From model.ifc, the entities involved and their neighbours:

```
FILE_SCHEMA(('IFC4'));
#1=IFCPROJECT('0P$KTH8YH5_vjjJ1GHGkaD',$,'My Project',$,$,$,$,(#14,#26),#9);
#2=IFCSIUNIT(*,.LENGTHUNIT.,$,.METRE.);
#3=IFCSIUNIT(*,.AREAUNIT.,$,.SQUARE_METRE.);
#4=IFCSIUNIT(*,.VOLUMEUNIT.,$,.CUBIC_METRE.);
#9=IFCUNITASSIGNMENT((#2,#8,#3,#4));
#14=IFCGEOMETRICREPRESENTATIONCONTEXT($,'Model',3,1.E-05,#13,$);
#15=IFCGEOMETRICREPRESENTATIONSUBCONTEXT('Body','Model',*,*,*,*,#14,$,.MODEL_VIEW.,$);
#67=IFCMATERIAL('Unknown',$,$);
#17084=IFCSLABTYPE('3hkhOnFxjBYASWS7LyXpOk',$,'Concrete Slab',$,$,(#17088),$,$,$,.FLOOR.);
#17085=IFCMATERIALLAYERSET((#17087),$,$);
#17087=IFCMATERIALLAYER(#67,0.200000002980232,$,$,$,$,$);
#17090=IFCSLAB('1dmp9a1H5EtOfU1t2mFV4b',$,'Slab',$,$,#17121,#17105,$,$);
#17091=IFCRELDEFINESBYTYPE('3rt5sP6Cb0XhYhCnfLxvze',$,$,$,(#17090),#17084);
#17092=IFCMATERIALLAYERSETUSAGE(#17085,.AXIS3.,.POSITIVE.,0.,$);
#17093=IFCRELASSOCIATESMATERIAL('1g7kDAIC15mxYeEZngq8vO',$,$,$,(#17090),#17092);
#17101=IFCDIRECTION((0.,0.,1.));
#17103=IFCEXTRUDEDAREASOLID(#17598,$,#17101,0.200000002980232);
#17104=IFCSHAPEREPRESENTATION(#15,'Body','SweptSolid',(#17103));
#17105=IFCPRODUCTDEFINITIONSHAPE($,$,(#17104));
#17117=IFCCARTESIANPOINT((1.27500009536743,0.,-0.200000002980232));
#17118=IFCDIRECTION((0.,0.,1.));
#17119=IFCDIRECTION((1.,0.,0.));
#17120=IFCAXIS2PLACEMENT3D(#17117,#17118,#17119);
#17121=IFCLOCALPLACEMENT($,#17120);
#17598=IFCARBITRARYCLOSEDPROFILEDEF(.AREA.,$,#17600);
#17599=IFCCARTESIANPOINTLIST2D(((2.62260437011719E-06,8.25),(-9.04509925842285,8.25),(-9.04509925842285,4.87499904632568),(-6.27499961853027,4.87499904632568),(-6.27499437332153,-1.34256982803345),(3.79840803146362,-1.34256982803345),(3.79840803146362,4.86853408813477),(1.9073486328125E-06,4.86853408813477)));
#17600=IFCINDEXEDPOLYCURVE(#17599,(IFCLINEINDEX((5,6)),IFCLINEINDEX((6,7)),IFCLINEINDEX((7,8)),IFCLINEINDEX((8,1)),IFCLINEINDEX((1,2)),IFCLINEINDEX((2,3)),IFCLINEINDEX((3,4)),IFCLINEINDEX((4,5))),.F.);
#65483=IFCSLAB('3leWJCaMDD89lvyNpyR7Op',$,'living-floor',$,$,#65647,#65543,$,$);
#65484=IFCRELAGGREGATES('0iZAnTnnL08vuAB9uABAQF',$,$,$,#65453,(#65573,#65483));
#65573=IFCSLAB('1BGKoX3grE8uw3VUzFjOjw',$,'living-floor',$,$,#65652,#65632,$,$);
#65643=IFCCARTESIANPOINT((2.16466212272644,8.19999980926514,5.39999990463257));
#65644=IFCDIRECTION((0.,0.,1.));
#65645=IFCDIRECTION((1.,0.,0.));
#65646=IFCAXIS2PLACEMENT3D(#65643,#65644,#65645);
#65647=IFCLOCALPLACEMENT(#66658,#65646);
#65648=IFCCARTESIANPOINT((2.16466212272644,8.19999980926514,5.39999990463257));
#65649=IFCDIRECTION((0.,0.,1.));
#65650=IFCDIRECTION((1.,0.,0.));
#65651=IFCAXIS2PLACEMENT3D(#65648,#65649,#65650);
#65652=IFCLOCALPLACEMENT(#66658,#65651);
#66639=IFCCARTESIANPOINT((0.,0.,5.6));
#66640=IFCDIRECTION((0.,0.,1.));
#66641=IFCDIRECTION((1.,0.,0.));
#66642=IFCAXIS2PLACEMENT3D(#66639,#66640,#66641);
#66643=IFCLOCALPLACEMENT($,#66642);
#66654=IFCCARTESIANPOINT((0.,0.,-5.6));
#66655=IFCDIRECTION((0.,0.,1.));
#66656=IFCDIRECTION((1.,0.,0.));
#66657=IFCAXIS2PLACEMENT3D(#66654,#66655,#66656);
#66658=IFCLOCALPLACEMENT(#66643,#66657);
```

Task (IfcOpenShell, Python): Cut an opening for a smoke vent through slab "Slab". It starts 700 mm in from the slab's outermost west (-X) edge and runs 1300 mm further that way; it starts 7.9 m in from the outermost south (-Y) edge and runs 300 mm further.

```python
import numpy as np
import ifcopenshell
import ifcopenshell.api.feature
import ifcopenshell.api.geometry
import ifcopenshell.api.root
import ifcopenshell.geom
import ifcopenshell.util.placement
import ifcopenshell.util.representation
import ifcopenshell.util.shape
import ifcopenshell.util.unit

model = ifcopenshell.open("model.ifc")
unit_scale = ifcopenshell.util.unit.calculate_unit_scale(model)
settings = ifcopenshell.geom.settings()


def volume(element):
    """Net volume in cubic metres, openings subtracted."""
    shape = ifcopenshell.geom.create_shape(settings, element)
    return ifcopenshell.util.shape.get_volume(shape.geometry)


slab = model.by_guid("1dmp9a1H5EtOfU1t2mFV4b")
before = volume(slab)

# Extent in the slab's own axes, in metres. The edges named are its -X and -Y sides.
slab_shape = ifcopenshell.geom.create_shape(settings, slab)
vertices = ifcopenshell.util.shape.get_vertices(slab_shape.geometry)
x_min, y_min, bottom = vertices.min(axis=0)
top = vertices[:, 2].max()

opening = ifcopenshell.api.root.create_entity(model, ifc_class="IfcOpeningElement", name="Smoke vent opening", predefined_type="OPENING")
context = ifcopenshell.util.representation.get_context(model, "Model", "Body", "MODEL_VIEW")
width, depth = 1.3, 0.3
outline = [(0.0, 0.0), (width, 0.0), (width, depth), (0.0, depth), (0.0, 0.0)]
# Overshoot both faces by 50 mm so the cut is clean.
shape = ifcopenshell.api.geometry.add_slab_representation(
    model, context=context, depth=top - bottom + 0.1, polyline=outline
)
ifcopenshell.api.geometry.assign_representation(model, product=opening, representation=shape)

matrix = ifcopenshell.util.placement.get_local_placement(slab.ObjectPlacement)
matrix[:, 3] = matrix @ np.append(np.array([x_min + 0.7, y_min + 7.9, bottom - 0.05]) / unit_scale, 1.0)
ifcopenshell.api.geometry.edit_object_placement(model, product=opening, matrix=matrix, is_si=False)
ifcopenshell.api.feature.add_feature(model, feature=opening, element=slab)

after = volume(slab)

print(f"slab volume {before:.3f} -> {after:.3f} m3")

model.write("model_edited.ifc")
```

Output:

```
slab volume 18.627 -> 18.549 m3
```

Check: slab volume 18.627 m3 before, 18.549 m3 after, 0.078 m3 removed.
